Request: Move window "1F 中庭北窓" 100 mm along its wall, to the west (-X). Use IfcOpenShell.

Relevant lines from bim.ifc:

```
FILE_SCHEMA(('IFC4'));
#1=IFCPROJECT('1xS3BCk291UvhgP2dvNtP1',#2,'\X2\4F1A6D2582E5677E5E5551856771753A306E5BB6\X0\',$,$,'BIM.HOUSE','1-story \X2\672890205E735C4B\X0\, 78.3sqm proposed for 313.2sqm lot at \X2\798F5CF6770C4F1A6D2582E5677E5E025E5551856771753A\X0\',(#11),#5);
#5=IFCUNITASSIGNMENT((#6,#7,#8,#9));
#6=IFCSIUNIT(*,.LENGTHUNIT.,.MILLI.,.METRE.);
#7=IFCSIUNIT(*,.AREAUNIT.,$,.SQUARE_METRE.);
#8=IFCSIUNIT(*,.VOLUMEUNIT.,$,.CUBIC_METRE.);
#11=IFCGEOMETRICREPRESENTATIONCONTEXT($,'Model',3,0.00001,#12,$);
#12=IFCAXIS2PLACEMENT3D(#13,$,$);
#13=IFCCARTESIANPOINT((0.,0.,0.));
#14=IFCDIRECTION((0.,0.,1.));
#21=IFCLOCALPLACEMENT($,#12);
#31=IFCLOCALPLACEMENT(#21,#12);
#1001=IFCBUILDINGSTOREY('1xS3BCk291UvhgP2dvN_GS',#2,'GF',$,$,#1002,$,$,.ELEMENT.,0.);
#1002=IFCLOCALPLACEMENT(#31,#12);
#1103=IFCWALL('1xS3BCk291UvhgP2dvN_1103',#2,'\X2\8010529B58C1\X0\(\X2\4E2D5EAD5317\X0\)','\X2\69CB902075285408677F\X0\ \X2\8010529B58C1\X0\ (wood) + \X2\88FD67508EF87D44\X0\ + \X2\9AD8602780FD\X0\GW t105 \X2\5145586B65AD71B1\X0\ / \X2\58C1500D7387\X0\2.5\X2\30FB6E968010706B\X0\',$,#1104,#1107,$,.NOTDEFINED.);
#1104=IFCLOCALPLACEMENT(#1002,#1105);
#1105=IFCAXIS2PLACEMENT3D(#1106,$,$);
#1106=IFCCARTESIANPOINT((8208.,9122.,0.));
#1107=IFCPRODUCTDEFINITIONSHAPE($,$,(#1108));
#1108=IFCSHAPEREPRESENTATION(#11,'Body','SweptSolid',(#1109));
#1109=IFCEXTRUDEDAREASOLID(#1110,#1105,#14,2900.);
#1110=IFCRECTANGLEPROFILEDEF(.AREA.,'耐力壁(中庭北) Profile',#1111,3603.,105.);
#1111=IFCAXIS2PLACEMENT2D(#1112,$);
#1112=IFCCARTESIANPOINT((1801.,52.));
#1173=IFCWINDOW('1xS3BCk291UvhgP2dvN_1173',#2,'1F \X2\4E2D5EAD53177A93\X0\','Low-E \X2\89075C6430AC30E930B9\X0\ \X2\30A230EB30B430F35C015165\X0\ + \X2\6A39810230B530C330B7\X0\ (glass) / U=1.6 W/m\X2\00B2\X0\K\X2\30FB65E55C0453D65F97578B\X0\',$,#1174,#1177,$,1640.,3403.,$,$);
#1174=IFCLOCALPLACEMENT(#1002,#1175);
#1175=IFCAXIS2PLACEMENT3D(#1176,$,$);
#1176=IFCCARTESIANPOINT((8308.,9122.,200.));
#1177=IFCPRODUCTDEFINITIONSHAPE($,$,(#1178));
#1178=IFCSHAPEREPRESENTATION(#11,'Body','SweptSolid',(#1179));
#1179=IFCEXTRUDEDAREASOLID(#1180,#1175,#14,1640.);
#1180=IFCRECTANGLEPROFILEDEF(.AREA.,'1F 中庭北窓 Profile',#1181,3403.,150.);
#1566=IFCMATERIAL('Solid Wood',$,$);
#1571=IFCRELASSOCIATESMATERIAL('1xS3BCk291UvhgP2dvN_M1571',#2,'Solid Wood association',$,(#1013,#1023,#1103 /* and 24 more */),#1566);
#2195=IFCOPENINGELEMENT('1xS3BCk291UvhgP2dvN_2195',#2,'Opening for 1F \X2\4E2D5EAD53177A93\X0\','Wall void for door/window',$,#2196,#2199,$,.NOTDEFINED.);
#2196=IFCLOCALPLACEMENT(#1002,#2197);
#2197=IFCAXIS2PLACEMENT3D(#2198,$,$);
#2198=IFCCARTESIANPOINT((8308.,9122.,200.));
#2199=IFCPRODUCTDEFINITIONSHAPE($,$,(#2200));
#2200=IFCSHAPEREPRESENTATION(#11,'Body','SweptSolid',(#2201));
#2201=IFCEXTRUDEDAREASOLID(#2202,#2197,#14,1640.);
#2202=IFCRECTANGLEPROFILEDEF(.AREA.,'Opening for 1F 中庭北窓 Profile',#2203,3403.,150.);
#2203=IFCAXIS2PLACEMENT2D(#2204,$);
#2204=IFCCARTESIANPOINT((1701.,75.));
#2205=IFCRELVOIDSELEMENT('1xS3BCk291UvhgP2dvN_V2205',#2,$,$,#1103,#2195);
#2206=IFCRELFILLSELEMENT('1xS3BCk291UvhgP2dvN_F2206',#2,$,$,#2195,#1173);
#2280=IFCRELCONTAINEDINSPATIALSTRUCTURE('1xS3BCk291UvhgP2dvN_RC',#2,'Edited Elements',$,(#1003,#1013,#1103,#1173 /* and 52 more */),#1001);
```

```python
import ifcopenshell
import ifcopenshell.api.geometry
import ifcopenshell.util.placement
import ifcopenshell.util.unit

model = ifcopenshell.open("bim.ifc")
unit_scale = ifcopenshell.util.unit.calculate_unit_scale(model)

window = model.by_guid("1xS3BCk291UvhgP2dvN_1173")
opening = window.FillsVoids[0].RelatingOpeningElement
wall = opening.VoidsElements[0].RelatingBuildingElement

wall_matrix = ifcopenshell.util.placement.get_local_placement(wall.ObjectPlacement)
shift = wall_matrix[:3, 0] * -0.1 / unit_scale
before = ifcopenshell.util.placement.get_local_placement(window.ObjectPlacement)[:3, 3].copy()

# The window is not placed relative to its opening, so move both.
for product in (opening, window):
    matrix = ifcopenshell.util.placement.get_local_placement(product.ObjectPlacement)
    matrix[:3, 3] += shift
    ifcopenshell.api.geometry.edit_object_placement(model, product=product, matrix=matrix, is_si=False)

after = ifcopenshell.util.placement.get_local_placement(window.ObjectPlacement)[:3, 3]
print("window moved by", (after - before).round(3) + 0.0)

model.write("bim_edited.ifc")
```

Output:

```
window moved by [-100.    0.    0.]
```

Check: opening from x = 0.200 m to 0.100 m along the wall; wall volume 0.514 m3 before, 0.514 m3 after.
